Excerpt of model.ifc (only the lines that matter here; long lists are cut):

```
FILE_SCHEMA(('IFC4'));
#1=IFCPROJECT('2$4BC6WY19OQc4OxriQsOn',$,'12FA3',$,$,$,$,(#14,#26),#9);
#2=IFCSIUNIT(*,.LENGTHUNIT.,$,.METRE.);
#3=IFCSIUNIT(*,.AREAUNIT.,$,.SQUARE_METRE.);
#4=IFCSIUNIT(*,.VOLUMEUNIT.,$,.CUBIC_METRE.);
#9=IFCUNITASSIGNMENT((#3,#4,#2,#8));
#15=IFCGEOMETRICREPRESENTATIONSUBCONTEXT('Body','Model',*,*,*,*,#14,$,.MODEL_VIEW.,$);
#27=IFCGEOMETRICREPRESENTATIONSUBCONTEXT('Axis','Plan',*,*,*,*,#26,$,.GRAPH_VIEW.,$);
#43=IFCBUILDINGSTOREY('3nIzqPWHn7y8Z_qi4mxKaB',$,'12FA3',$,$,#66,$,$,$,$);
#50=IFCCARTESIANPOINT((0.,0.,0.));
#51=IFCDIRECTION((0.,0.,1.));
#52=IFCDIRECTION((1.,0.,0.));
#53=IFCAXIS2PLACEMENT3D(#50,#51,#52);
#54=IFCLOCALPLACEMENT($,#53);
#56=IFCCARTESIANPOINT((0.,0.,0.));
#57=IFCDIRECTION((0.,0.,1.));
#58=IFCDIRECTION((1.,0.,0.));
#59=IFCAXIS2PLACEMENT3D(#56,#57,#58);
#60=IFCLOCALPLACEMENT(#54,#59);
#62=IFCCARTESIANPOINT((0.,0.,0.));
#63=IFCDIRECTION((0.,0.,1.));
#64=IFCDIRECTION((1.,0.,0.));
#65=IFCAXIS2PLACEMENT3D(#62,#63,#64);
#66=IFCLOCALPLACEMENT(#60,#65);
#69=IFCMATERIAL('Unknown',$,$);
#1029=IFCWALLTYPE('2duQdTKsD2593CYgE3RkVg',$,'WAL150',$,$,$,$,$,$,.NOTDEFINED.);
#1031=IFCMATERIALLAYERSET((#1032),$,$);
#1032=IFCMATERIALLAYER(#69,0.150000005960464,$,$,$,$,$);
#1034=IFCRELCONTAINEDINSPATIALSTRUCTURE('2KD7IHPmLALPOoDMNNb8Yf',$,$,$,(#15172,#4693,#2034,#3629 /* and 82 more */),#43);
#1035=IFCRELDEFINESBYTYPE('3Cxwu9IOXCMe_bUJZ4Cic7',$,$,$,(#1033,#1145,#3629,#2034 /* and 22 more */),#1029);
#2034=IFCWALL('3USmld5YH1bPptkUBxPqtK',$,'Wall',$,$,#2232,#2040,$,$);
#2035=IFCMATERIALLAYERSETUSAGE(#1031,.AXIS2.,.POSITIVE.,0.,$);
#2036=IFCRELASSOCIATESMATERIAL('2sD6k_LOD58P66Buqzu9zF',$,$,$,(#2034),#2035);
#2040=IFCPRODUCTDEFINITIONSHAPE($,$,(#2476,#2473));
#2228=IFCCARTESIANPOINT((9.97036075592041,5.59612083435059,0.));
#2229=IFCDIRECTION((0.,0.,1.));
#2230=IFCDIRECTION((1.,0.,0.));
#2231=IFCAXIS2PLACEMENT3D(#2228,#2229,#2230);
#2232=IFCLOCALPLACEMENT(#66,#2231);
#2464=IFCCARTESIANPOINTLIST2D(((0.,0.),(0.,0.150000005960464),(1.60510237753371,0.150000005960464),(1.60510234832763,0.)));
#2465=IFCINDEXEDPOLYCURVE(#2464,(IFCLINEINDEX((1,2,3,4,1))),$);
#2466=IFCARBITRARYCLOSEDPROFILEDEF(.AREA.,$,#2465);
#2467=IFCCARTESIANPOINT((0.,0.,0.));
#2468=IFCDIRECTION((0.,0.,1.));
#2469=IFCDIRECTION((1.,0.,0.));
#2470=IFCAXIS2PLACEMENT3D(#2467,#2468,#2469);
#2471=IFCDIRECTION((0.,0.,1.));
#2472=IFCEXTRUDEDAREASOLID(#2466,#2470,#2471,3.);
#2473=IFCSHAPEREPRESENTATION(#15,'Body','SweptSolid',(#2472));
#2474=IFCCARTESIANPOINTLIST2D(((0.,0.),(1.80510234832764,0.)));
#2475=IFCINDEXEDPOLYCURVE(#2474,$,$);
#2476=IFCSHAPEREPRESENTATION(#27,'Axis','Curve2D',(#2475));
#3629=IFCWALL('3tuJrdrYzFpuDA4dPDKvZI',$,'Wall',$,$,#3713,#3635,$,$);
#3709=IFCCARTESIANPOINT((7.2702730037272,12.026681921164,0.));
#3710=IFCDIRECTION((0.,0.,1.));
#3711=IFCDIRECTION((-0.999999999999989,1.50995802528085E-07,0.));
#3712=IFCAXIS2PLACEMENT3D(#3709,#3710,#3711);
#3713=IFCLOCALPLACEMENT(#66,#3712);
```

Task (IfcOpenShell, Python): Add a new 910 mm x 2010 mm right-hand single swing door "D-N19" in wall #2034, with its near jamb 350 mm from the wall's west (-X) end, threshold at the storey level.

```python
import numpy as np
import ifcopenshell
import ifcopenshell.api.feature
import ifcopenshell.api.geometry
import ifcopenshell.api.root
import ifcopenshell.api.spatial
import ifcopenshell.geom
import ifcopenshell.util.element
import ifcopenshell.util.placement
import ifcopenshell.util.representation
import ifcopenshell.util.shape
import ifcopenshell.util.unit

model = ifcopenshell.open("model.ifc")
unit_scale = ifcopenshell.util.unit.calculate_unit_scale(model)
settings = ifcopenshell.geom.settings()


def volume(element):
    """Net volume in cubic metres, openings subtracted."""
    shape = ifcopenshell.geom.create_shape(settings, element)
    return ifcopenshell.util.shape.get_volume(shape.geometry)


wall = model.by_guid("3USmld5YH1bPptkUBxPqtK")
storey = ifcopenshell.util.element.get_container(wall, ifc_class="IfcBuildingStorey")
context = ifcopenshell.util.representation.get_context(model, "Model", "Body", "MODEL_VIEW")
before = volume(wall)

width, height, from_end, sill = 0.91, 2.01, 0.35, 0.0  # metres

# The wall runs along its own X axis, and the end named is its -X end.
wall_shape = ifcopenshell.geom.create_shape(settings, wall)
x, y, z = ifcopenshell.util.shape.get_vertices(wall_shape.geometry).T
start = x.min() + from_end
face, thickness = float(y.min()), float(y.max() - y.min())
wall_matrix = ifcopenshell.util.placement.get_local_placement(wall.ObjectPlacement)
level = ifcopenshell.util.placement.get_local_placement(storey.ObjectPlacement)[2, 3]


def in_wall(x, y):
    """Placement at x, y metres in the wall's axes, at sill height."""
    matrix = wall_matrix.copy()
    matrix[:, 3] = wall_matrix @ np.array([x / unit_scale, y / unit_scale, 0.0, 1.0])
    matrix[2, 3] = level + sill / unit_scale
    return matrix


# Opening: a box that overshoots both wall faces by 50 mm.
opening = ifcopenshell.api.root.create_entity(model, ifc_class="IfcOpeningElement", predefined_type="OPENING")
box = ifcopenshell.api.geometry.add_wall_representation(
    model, context=context, length=width, height=height, thickness=thickness + 0.1
)
ifcopenshell.api.geometry.assign_representation(model, product=opening, representation=box)
ifcopenshell.api.geometry.edit_object_placement(model, product=opening, matrix=in_wall(start, face - 0.05), is_si=False)
ifcopenshell.api.feature.add_feature(model, feature=opening, element=wall)

door = ifcopenshell.api.root.create_entity(model, ifc_class="IfcDoor", name="D-N19", predefined_type="DOOR")
door.OverallWidth, door.OverallHeight = width / unit_scale, height / unit_scale
door.OperationType = "SINGLE_SWING_RIGHT"
body = ifcopenshell.api.geometry.add_door_representation(
    model,
    context=context,
    overall_width=door.OverallWidth,
    overall_height=door.OverallHeight,
    operation_type="SINGLE_SWING_RIGHT",
    lining_properties={"LiningDepth": thickness / unit_scale, "ThresholdDepth": thickness / unit_scale},
)
ifcopenshell.api.geometry.assign_representation(model, product=door, representation=body)
ifcopenshell.api.spatial.assign_container(model, products=[door], relating_structure=storey)
ifcopenshell.api.feature.add_filling(model, opening=opening, element=door)

# The lining spans the wall, so the door starts at the wall face.
ifcopenshell.api.geometry.edit_object_placement(model, product=door, matrix=in_wall(start, face), is_si=False)

after = volume(wall)

print(f"wall volume {before:.3f} -> {after:.3f} m3")

model.write("model_edited.ifc")
```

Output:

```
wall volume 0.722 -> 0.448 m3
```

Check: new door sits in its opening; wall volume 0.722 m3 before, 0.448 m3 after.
